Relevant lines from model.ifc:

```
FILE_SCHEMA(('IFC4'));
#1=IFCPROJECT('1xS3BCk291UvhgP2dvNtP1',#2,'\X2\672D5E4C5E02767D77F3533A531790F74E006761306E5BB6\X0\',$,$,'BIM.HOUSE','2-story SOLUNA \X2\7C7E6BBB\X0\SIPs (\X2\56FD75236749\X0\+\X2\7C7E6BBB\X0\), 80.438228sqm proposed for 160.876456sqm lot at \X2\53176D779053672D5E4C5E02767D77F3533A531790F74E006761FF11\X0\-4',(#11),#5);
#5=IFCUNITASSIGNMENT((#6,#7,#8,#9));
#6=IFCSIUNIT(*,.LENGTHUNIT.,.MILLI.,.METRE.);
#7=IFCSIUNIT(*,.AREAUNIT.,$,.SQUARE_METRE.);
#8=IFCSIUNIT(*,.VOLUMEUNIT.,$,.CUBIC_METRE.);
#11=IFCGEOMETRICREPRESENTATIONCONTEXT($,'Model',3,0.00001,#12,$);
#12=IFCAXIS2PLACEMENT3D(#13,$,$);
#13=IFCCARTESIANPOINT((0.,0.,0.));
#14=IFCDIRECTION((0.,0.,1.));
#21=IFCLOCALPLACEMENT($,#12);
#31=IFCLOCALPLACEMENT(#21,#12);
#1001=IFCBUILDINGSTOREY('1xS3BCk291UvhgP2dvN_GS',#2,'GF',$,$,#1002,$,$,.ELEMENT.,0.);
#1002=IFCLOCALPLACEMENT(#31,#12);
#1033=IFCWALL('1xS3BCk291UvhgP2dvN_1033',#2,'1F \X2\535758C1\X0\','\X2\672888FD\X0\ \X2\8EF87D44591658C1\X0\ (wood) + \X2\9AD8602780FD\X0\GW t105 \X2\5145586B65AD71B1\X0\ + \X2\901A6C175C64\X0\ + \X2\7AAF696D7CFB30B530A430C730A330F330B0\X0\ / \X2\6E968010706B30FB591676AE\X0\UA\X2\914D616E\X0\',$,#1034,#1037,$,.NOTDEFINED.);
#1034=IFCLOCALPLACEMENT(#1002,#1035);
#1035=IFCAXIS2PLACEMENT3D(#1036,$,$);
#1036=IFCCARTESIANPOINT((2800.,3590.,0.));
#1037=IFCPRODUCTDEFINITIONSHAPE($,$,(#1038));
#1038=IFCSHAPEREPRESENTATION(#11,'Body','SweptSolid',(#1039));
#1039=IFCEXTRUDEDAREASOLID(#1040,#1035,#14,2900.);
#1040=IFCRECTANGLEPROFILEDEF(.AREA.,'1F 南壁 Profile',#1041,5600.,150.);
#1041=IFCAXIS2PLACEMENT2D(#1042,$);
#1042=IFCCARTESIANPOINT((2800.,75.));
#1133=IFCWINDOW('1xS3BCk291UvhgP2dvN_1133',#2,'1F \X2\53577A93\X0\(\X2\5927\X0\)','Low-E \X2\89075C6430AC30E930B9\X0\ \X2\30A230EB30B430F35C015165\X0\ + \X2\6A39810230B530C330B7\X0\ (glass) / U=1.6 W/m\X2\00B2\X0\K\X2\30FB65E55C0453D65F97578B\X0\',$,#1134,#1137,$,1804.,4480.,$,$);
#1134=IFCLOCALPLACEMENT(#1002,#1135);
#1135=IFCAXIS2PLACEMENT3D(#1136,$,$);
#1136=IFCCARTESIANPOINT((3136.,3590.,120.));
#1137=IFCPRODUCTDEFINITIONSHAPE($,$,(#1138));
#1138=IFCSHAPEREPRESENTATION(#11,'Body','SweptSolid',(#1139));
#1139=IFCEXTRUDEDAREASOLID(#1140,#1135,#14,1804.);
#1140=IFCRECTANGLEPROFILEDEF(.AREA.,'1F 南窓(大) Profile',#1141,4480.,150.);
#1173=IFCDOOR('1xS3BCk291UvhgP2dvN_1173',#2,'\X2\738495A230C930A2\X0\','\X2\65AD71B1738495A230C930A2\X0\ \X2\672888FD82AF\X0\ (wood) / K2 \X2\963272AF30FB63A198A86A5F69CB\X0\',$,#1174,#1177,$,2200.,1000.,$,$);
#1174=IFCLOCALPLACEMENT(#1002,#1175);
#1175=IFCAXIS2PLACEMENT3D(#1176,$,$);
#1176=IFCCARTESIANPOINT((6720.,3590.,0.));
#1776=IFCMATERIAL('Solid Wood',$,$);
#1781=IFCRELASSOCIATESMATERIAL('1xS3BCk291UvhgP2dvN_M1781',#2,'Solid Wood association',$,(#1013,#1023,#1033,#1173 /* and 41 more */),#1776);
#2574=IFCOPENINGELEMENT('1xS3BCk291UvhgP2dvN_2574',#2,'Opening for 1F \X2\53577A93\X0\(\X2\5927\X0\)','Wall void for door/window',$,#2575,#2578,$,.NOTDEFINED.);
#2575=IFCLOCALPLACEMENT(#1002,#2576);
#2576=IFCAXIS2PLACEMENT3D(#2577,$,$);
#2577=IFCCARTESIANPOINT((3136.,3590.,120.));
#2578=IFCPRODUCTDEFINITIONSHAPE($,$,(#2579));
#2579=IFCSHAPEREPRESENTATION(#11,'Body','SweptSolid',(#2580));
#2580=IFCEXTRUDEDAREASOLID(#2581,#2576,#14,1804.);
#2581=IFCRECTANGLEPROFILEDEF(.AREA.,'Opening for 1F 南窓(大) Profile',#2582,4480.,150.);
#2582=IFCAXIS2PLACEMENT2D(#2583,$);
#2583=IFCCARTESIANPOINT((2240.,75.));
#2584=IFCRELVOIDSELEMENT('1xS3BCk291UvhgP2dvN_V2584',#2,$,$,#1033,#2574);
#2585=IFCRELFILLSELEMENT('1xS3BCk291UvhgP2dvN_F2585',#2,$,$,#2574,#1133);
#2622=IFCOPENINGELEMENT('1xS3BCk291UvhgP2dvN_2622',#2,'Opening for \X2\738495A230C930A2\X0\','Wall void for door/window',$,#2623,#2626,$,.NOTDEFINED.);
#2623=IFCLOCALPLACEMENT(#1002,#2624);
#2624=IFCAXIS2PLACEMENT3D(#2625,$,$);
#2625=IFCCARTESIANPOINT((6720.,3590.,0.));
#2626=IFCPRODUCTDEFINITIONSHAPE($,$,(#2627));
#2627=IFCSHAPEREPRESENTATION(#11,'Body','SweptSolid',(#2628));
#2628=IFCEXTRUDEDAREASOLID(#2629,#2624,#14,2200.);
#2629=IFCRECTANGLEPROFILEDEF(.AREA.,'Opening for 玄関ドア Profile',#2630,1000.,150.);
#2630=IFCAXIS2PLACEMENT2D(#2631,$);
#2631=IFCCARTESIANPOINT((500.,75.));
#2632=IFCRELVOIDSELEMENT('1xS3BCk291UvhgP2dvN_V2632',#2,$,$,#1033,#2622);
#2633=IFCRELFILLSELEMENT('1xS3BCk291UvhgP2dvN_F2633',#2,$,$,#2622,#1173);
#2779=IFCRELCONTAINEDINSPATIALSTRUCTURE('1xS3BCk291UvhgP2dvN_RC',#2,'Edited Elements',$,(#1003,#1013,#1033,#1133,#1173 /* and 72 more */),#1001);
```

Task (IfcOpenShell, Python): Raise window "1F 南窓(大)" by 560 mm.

```python
import numpy as np
import ifcopenshell
import ifcopenshell.api.geometry
import ifcopenshell.util.placement
import ifcopenshell.util.unit

model = ifcopenshell.open("model.ifc")
unit_scale = ifcopenshell.util.unit.calculate_unit_scale(model)

window = model.by_guid("1xS3BCk291UvhgP2dvN_1133")
opening = window.FillsVoids[0].RelatingOpeningElement
dz = 560.0

shift = np.array([0.0, 0.0, dz])
# The window is not placed relative to its opening, so move both.
for product in (opening, window):
    matrix = ifcopenshell.util.placement.get_local_placement(product.ObjectPlacement)
    matrix[:3, 3] += shift
    ifcopenshell.api.geometry.edit_object_placement(model, product=product, matrix=matrix, is_si=False)

print(f"moved by {dz * unit_scale:+.3f} m")

model.write("model-out.ifc")
```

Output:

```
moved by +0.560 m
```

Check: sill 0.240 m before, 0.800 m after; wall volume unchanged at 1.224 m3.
